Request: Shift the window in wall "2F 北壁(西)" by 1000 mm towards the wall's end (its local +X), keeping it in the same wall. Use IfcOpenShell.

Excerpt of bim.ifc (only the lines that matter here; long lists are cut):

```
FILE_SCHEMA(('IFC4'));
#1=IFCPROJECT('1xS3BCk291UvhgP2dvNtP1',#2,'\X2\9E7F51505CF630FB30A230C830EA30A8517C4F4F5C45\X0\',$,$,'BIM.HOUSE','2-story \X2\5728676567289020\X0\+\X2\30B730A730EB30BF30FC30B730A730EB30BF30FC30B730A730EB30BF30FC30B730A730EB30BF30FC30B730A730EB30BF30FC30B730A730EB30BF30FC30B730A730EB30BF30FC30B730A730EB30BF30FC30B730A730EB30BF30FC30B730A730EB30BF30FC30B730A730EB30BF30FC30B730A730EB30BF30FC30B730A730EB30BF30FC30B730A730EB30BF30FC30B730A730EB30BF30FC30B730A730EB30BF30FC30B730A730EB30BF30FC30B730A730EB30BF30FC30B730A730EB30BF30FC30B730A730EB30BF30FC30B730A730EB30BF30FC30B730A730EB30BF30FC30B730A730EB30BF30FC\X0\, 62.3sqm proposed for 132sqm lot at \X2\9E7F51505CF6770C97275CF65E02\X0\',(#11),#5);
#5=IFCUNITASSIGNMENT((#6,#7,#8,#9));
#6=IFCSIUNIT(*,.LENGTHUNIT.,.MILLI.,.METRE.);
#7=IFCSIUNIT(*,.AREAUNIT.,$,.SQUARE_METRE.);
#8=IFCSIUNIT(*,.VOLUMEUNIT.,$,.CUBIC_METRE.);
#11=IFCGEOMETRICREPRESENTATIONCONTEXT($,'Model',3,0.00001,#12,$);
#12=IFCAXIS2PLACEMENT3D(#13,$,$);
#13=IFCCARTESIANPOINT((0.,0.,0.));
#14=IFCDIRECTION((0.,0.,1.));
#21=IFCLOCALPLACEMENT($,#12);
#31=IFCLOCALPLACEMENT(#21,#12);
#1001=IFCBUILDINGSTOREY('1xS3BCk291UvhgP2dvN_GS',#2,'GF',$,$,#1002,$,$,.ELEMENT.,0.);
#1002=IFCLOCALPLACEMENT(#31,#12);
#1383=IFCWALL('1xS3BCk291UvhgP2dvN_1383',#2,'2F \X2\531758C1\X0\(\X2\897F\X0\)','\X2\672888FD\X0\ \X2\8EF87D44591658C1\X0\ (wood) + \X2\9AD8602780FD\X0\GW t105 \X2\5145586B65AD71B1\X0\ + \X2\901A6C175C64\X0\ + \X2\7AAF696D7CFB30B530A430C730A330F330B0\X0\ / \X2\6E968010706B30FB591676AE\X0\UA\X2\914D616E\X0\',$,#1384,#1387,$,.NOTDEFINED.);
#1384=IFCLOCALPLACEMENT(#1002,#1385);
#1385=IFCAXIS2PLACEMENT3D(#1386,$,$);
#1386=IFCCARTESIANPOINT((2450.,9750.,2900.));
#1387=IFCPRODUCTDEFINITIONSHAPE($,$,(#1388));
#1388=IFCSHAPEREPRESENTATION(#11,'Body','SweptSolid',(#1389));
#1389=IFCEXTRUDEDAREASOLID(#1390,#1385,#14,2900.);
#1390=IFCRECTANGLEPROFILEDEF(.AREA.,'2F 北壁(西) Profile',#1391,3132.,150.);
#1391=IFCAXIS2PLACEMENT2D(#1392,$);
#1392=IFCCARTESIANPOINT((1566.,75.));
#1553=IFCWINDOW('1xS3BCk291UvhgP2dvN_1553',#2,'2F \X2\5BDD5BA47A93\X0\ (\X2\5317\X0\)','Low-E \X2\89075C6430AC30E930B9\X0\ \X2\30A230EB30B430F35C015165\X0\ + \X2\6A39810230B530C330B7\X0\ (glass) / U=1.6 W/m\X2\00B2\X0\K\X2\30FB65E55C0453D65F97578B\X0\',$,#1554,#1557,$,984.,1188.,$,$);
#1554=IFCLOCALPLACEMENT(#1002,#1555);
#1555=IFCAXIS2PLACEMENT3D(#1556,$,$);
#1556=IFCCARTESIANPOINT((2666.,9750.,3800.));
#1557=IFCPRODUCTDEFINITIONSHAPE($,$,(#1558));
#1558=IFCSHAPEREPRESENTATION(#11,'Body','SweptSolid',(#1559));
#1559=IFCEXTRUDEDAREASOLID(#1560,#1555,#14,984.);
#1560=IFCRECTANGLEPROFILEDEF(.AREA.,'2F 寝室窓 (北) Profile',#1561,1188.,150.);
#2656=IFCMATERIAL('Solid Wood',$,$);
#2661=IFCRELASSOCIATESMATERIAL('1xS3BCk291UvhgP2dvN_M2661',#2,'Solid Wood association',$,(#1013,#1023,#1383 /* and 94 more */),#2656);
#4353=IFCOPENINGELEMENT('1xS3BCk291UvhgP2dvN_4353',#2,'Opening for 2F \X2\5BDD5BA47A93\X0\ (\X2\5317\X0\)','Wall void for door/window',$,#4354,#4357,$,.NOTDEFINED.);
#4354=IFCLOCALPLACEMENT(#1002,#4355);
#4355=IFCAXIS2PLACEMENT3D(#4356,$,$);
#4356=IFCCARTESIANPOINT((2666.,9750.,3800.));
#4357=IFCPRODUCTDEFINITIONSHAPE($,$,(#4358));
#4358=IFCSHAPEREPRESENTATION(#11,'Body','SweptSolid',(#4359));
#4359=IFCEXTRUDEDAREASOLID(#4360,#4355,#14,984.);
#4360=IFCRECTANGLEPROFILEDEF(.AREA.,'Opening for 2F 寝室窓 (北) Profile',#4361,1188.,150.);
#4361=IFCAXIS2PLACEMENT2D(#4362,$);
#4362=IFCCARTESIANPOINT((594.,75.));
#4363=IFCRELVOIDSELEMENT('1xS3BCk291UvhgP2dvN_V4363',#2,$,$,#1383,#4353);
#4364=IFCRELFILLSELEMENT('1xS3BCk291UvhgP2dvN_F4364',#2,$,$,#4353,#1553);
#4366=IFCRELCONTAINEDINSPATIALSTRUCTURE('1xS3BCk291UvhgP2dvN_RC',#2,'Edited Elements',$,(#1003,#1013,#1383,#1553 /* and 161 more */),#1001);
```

```python
import ifcopenshell
import ifcopenshell.api.geometry
import ifcopenshell.util.placement

model = ifcopenshell.open("bim.ifc")

window = model.by_guid("1xS3BCk291UvhgP2dvN_1553")
opening = window.FillsVoids[0].RelatingOpeningElement
wall = opening.VoidsElements[0].RelatingBuildingElement

wall_matrix = ifcopenshell.util.placement.get_local_placement(wall.ObjectPlacement)
shift = wall_matrix[:3, 0] * 1000.0
before = ifcopenshell.util.placement.get_local_placement(window.ObjectPlacement)[:3, 3].copy()

# The window is not placed relative to its opening, so move both.
for product in (opening, window):
    matrix = ifcopenshell.util.placement.get_local_placement(product.ObjectPlacement)
    matrix[:3, 3] += shift
    ifcopenshell.api.geometry.edit_object_placement(model, product=product, matrix=matrix, is_si=False)

after = ifcopenshell.util.placement.get_local_placement(window.ObjectPlacement)[:3, 3]
print("window moved by", (after - before).round(3) + 0.0)

model.write("bim_edited.ifc")
```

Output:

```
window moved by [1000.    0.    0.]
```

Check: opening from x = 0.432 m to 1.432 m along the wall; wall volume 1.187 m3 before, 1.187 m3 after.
